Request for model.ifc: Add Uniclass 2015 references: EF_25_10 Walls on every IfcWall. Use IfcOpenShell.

First a look at what the model holds.

```python
import ifcopenshell

model = ifcopenshell.open("model.ifc")
print(model.schema)
print("classifications:", [c.Name for c in model.by_type("IfcClassification")])
for ifc_class in ("IfcDoor", "IfcRoof", "IfcStair", "IfcWall", "IfcWindow"):
    print(ifc_class, len(model.by_type(ifc_class)))
```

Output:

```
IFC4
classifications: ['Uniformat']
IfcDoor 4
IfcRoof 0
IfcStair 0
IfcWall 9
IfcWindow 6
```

```python
import ifcopenshell
import ifcopenshell.api.classification

model = ifcopenshell.open("model.ifc")

system = ifcopenshell.api.classification.add_classification(model, classification="Uniclass 2015")

codes = {
    "IfcWall": ("EF_25_10", "Walls"),
}
for ifc_class, (code, name) in codes.items():
    products = model.by_type(ifc_class)
    ifcopenshell.api.classification.add_reference(
        model, products=products, classification=system, identification=code, name=name
    )
    print(code, len(products))

model.write("model-out.ifc")
```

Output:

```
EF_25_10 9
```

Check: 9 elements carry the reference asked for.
